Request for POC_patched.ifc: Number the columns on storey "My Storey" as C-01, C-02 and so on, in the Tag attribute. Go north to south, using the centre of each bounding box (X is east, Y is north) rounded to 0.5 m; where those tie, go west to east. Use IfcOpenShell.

First a look at what the model holds.

```python
import ifcopenshell
import ifcopenshell.util.element
import ifcopenshell.util.placement

model = ifcopenshell.open("POC_patched.ifc")
print(model.schema)
storey = next(s for s in model.by_type("IfcBuildingStorey") if s.Name == "My Storey")
columns = [e for e in ifcopenshell.util.element.get_decomposition(storey) if e.is_a("IfcColumn")]
for e in sorted(columns, key=lambda e: e.id()):
    origin = ifcopenshell.util.placement.get_local_placement(e.ObjectPlacement)[:3, 3]
    print(e.id(), e.Tag, e.Name, origin.round(2) + 0.0, sep=" | ")
```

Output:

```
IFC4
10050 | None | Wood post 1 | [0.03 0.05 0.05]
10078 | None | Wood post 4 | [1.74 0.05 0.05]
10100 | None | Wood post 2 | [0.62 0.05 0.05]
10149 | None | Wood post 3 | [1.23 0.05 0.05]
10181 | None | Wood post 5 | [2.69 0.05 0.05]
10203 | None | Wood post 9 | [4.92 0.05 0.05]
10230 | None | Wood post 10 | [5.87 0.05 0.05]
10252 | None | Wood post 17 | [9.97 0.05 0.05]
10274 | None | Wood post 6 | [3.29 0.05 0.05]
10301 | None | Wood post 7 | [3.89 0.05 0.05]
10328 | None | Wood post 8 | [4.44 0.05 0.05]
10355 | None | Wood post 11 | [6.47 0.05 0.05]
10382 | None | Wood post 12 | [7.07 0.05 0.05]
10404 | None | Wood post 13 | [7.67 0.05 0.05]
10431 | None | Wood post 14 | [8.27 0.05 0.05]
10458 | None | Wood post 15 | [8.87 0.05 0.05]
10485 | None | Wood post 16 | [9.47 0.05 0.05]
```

```python
import ifcopenshell
import ifcopenshell.geom
import ifcopenshell.util.element
import ifcopenshell.util.shape

model = ifcopenshell.open("POC_patched.ifc")
settings = ifcopenshell.geom.settings()
settings.set("use-world-coords", True)


def centre(element):
    shape = ifcopenshell.geom.create_shape(settings, element)
    return ifcopenshell.util.shape.get_bbox_centroid(shape.geometry)


storey = next(s for s in model.by_type("IfcBuildingStorey") if s.Name == "My Storey")
columns = [e for e in ifcopenshell.util.element.get_decomposition(storey) if e.is_a("IfcColumn")]

# Insertion points can sit at a corner or the storey origin, so sort by the geometry (in metres).
centres = {e: centre(e) for e in columns}
columns.sort(key=lambda e: (-round(centres[e][1] / 0.5), centres[e][0]))

for i, e in enumerate(columns, start=1):
    number = f"C-{i:02d}"
    e.Tag = number
    print(e.id(), number)

model.write("POC_patched_rev.ifc")
```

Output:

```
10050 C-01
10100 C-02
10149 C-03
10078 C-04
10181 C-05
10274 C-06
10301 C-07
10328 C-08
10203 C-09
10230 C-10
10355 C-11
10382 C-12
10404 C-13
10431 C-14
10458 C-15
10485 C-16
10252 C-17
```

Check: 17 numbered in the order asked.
